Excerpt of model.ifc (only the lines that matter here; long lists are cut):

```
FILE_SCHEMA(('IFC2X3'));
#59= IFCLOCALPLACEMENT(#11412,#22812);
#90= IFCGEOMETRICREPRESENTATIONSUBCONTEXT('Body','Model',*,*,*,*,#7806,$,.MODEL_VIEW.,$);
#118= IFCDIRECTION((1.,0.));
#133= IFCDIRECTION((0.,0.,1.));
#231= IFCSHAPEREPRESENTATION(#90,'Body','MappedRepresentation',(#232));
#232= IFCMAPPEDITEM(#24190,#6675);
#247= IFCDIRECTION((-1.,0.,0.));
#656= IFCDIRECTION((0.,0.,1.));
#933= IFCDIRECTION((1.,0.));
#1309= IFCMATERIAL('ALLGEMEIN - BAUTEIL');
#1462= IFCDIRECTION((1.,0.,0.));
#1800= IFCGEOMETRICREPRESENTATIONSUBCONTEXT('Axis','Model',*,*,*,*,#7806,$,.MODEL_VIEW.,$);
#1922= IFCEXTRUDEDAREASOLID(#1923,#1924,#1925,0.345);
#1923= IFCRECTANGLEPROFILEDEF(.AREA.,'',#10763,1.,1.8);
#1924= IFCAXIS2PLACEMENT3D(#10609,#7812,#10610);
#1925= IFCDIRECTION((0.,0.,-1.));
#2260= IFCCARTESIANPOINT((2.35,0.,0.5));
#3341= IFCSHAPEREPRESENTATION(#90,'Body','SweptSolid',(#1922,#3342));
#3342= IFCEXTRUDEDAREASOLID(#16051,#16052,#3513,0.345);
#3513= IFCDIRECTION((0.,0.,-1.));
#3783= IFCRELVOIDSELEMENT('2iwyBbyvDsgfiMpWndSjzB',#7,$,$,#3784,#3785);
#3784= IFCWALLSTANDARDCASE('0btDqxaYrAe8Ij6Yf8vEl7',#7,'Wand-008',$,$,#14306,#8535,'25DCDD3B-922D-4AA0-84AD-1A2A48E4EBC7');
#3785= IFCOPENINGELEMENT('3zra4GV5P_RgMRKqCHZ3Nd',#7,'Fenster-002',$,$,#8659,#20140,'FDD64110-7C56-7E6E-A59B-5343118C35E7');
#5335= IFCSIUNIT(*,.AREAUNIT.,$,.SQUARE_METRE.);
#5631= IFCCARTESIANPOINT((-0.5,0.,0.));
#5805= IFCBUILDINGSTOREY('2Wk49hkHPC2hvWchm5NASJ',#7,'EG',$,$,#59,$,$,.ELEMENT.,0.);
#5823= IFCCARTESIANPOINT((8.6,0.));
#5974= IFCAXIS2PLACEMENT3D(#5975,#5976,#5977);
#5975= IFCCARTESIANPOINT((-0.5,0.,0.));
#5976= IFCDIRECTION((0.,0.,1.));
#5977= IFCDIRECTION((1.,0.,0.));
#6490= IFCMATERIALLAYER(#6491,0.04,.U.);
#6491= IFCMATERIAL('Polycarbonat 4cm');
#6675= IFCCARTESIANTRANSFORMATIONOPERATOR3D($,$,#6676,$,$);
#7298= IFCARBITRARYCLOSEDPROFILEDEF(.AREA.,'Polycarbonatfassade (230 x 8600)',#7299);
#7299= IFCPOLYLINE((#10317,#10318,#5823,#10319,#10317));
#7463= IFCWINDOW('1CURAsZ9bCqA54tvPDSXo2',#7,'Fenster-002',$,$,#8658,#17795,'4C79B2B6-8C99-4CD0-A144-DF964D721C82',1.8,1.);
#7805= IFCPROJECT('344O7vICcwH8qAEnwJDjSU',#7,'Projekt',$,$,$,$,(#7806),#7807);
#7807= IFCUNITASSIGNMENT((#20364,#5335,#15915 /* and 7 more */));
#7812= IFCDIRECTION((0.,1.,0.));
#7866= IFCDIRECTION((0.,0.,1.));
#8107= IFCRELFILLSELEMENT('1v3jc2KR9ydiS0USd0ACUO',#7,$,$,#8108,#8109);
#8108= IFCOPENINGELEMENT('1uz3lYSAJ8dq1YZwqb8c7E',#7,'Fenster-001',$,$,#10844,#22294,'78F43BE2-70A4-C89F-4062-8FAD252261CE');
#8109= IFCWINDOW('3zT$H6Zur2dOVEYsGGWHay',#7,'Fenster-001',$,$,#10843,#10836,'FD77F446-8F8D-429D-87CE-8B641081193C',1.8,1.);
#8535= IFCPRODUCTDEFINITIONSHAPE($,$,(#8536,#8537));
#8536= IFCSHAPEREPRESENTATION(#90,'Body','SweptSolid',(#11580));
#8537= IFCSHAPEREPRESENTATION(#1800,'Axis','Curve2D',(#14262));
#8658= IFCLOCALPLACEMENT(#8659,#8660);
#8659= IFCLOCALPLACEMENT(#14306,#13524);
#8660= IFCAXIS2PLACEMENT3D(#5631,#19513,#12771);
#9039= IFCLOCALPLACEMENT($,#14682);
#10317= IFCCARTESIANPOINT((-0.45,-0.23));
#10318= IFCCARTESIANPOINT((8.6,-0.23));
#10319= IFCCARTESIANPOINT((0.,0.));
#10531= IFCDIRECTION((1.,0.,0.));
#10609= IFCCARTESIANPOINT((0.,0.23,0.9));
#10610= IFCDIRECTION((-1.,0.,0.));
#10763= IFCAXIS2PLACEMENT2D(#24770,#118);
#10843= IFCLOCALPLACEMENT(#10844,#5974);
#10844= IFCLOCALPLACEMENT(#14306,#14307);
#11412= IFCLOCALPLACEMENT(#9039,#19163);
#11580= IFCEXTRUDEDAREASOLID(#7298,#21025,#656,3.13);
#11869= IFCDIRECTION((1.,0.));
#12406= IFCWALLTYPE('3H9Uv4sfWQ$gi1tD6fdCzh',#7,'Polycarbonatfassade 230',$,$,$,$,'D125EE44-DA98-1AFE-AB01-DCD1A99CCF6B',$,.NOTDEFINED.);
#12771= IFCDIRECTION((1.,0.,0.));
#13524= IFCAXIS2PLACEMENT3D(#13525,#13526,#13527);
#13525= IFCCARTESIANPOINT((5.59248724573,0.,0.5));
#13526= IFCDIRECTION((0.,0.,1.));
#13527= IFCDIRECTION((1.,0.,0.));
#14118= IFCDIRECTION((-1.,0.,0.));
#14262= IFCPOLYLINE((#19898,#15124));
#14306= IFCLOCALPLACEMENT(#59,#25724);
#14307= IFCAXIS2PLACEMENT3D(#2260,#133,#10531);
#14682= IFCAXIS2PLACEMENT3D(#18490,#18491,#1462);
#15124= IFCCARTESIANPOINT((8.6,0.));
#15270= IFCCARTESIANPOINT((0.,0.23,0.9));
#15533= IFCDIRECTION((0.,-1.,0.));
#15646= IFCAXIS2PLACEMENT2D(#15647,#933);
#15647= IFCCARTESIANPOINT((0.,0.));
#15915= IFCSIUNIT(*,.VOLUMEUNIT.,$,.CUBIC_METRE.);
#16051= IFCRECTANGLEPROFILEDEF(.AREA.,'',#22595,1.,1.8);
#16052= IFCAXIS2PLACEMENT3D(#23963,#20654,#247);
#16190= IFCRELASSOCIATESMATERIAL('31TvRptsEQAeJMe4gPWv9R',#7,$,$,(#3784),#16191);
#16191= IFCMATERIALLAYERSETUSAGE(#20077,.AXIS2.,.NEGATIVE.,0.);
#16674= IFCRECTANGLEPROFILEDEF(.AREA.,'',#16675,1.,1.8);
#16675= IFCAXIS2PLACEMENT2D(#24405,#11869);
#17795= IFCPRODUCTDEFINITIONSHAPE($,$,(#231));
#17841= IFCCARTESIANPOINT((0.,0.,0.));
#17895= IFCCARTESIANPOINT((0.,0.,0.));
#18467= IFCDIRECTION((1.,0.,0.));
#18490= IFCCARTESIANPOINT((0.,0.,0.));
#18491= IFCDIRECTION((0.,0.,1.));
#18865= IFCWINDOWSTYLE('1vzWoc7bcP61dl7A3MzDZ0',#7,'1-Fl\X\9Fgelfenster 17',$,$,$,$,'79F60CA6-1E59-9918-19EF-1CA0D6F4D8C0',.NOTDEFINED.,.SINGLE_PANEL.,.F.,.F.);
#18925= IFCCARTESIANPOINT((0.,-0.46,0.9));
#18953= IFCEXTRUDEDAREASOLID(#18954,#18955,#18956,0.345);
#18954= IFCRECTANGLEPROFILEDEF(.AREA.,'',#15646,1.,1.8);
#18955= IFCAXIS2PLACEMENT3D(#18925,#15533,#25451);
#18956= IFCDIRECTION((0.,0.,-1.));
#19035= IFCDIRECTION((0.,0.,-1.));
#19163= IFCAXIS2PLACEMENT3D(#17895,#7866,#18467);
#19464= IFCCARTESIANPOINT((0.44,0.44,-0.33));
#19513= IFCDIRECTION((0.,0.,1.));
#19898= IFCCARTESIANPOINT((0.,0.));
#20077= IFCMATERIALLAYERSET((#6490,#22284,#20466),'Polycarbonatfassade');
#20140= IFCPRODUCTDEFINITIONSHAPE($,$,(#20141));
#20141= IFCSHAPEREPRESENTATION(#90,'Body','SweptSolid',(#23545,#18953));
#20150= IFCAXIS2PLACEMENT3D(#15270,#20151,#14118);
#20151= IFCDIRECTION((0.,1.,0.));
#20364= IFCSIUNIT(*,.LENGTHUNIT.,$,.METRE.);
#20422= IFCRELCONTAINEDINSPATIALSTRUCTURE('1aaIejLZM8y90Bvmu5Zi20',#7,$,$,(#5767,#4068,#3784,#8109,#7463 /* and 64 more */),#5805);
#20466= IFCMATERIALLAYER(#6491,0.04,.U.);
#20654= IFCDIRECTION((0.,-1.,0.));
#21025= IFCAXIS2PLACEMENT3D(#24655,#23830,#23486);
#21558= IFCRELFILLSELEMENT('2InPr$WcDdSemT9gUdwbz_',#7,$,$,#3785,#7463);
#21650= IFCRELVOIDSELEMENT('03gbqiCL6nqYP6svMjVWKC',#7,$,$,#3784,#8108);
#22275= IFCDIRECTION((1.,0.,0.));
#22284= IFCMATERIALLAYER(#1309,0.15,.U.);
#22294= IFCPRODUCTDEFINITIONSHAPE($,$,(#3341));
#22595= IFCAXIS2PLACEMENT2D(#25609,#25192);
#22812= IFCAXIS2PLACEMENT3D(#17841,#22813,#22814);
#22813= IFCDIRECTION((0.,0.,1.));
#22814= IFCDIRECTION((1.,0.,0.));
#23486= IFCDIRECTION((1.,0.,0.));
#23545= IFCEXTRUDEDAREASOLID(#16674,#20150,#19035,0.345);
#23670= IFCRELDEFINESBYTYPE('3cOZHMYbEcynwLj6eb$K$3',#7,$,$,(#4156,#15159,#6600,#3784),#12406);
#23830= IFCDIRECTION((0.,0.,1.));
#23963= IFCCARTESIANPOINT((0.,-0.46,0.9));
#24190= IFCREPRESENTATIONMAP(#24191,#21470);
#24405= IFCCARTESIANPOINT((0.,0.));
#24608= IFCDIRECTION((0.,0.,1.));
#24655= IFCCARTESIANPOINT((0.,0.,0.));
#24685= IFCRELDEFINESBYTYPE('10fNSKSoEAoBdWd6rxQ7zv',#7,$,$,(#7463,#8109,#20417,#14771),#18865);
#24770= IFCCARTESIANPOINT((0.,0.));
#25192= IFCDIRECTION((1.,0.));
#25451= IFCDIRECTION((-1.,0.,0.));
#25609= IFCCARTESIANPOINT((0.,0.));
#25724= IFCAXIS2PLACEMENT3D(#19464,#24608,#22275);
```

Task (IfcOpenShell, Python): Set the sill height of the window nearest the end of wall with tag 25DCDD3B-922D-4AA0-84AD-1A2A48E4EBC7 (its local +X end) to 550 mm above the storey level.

```python
import numpy as np
import ifcopenshell
import ifcopenshell.api.geometry
import ifcopenshell.geom
import ifcopenshell.util.element
import ifcopenshell.util.placement
import ifcopenshell.util.shape
import ifcopenshell.util.unit

model = ifcopenshell.open("model.ifc")
unit_scale = ifcopenshell.util.unit.calculate_unit_scale(model)

window = model.by_id(7463)
opening = window.FillsVoids[0].RelatingOpeningElement
storey = ifcopenshell.util.element.get_container(window, ifc_class="IfcBuildingStorey")
level = ifcopenshell.util.placement.get_local_placement(storey.ObjectPlacement)[2, 3]

# The opening's origin need not be at the sill, so measure its lowest point.
shape = ifcopenshell.geom.create_shape(ifcopenshell.geom.settings(), opening)
bottom = ifcopenshell.util.shape.get_shape_bottom_elevation(shape, shape.geometry) / unit_scale
dz = level + 0.55 / unit_scale - bottom

shift = np.array([0.0, 0.0, dz])
# The window is placed relative to its opening, so it follows when the opening moves.
matrix = ifcopenshell.util.placement.get_local_placement(opening.ObjectPlacement)
matrix[:3, 3] += shift
ifcopenshell.api.geometry.edit_object_placement(
    model, product=opening, matrix=matrix, is_si=False, should_transform_children=True
)

print(f"moved by {dz * unit_scale:+.3f} m")

model.write("model_edited.ifc")
```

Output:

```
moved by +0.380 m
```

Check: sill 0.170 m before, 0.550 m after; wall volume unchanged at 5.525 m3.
